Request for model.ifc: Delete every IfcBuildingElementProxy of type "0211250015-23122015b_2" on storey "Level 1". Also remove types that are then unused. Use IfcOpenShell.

First a look at what the model holds.

```python
import ifcopenshell
import ifcopenshell.util.element

model = ifcopenshell.open("model.ifc")
print(model.schema)
storey = next(s for s in model.by_type("IfcBuildingStorey") if s.Name == "Level 1")
proxies = [e for e in ifcopenshell.util.element.get_decomposition(storey) if e.is_a("IfcBuildingElementProxy")]
seen = {}
for e in proxies:
    element_type = ifcopenshell.util.element.get_type(e)
    name = element_type.Name if element_type not in (None, e) else None
    seen[name] = seen.get(name, 0) + 1
for name, count in sorted(seen.items(), key=str):
    print(count, "x", name)
```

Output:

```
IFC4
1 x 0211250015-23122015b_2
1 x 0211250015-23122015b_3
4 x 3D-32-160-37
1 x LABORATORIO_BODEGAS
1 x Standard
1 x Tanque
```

```python
import ifcopenshell
import ifcopenshell.api.root
import ifcopenshell.util.element

model = ifcopenshell.open("model.ifc")

storey = next(s for s in model.by_type("IfcBuildingStorey") if s.Name == "Level 1")
proxies = [e for e in ifcopenshell.util.element.get_decomposition(storey) if e.is_a("IfcBuildingElementProxy")]
targets = [e for e in proxies if (t := ifcopenshell.util.element.get_type(e)) not in (None, e) and t.Name == "0211250015-23122015b_2"]
types = {ifcopenshell.util.element.get_type(e) for e in targets} - {None, *targets}

for e in targets:
    ifcopenshell.api.root.remove_product(model, product=e)
print(len(targets), "removed")

unused = [t for t in types if not ifcopenshell.util.element.get_types(t)]
for t in unused:
    ifcopenshell.api.root.remove_product(model, product=t)
print(len(unused), "unused types removed")

model.write("model-out.ifc")
```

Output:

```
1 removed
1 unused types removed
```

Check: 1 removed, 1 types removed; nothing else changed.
